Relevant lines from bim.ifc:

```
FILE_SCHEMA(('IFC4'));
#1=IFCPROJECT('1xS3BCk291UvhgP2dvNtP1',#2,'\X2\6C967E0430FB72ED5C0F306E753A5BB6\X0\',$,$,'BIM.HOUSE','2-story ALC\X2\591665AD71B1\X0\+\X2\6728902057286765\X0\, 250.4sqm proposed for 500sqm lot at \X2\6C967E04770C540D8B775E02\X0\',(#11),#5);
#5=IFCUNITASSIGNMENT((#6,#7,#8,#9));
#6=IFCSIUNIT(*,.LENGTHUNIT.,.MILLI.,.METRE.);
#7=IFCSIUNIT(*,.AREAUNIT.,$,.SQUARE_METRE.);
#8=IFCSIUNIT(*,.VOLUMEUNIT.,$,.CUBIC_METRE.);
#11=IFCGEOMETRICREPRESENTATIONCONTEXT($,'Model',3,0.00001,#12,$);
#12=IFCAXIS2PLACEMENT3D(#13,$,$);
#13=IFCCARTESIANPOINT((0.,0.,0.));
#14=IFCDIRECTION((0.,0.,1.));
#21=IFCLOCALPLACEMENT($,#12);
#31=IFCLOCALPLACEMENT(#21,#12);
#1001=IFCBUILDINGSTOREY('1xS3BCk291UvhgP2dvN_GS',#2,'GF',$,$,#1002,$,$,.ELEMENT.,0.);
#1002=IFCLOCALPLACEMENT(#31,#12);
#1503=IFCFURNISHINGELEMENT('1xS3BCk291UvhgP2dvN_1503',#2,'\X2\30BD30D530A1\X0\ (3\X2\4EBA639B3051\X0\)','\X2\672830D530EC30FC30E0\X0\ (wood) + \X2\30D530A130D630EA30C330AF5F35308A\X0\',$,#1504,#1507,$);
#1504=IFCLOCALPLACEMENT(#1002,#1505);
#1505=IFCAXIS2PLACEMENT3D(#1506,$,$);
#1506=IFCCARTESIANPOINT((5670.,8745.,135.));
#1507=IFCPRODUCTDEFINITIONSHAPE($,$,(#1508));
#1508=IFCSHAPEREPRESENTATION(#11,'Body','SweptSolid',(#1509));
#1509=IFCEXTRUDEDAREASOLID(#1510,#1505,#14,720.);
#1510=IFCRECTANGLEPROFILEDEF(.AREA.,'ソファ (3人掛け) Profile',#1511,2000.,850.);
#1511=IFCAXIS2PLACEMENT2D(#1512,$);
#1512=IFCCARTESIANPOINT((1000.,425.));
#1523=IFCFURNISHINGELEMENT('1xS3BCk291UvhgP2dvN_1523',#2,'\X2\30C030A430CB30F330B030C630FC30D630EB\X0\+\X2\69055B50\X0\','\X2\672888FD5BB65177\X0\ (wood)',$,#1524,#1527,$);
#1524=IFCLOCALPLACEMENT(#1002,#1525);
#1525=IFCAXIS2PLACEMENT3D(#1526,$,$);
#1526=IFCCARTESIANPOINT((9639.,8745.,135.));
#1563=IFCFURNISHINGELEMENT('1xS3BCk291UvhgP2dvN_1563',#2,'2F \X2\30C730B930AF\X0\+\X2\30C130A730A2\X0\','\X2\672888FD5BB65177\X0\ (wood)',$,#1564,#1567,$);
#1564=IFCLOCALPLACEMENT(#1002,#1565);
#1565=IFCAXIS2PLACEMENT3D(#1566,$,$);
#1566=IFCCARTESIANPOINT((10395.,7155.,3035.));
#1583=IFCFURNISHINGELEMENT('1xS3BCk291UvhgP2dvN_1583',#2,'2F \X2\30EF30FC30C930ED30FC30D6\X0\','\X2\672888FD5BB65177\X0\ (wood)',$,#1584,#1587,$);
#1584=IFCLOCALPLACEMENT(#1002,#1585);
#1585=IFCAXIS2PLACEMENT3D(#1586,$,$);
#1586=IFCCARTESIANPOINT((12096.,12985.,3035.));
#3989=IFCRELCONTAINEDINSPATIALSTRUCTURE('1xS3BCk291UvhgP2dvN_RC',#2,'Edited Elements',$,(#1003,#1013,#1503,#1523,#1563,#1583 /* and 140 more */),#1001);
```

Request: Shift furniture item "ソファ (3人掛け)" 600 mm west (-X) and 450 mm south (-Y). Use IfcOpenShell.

```python
import ifcopenshell
import ifcopenshell.api.geometry
import ifcopenshell.util.placement
import ifcopenshell.util.unit

model = ifcopenshell.open("bim.ifc")
unit_scale = ifcopenshell.util.unit.calculate_unit_scale(model)

item = model.by_guid("1xS3BCk291UvhgP2dvN_1503")
matrix = ifcopenshell.util.placement.get_local_placement(item.ObjectPlacement)
matrix[0, 3] -= 0.6 / unit_scale
matrix[1, 3] -= 0.45 / unit_scale
ifcopenshell.api.geometry.edit_object_placement(model, product=item, matrix=matrix, is_si=False)

print(ifcopenshell.util.placement.get_local_placement(item.ObjectPlacement).round(3) + 0.0)

model.write("bim_updated.ifc")
```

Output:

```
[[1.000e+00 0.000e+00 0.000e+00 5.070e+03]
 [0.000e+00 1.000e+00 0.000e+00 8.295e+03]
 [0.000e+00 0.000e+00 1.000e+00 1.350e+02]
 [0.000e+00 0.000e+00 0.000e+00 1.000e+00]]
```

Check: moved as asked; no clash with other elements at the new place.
